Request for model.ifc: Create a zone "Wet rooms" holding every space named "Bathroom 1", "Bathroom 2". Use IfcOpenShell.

First a look at what the model holds.

```python
import ifcopenshell

model = ifcopenshell.open("model.ifc")
print(model.schema)
seen = {}
for space in model.by_type("IfcSpace"):
    seen[space.LongName] = seen.get(space.LongName, 0) + 1
for name, count in sorted(seen.items(), key=str):
    print(count, "x", name)
print("zones:", [z.Name for z in model.by_type("IfcZone")][:20])
```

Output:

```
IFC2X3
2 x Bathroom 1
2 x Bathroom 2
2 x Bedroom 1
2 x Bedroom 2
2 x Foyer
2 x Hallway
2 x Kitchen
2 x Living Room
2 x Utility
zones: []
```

```python
import ifcopenshell
import ifcopenshell.api.group
import ifcopenshell.api.root

model = ifcopenshell.open("model.ifc")

names = {"Bathroom 1", "Bathroom 2"}
spaces = [s for s in model.by_type("IfcSpace") if s.LongName in names]

zone = ifcopenshell.api.root.create_entity(model, ifc_class="IfcZone", name="Wet rooms")
ifcopenshell.api.group.assign_group(model, products=spaces, group=zone)
print(len(spaces), "spaces in", zone.Name)

model.write("model_updated.ifc")
```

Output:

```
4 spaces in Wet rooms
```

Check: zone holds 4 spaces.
